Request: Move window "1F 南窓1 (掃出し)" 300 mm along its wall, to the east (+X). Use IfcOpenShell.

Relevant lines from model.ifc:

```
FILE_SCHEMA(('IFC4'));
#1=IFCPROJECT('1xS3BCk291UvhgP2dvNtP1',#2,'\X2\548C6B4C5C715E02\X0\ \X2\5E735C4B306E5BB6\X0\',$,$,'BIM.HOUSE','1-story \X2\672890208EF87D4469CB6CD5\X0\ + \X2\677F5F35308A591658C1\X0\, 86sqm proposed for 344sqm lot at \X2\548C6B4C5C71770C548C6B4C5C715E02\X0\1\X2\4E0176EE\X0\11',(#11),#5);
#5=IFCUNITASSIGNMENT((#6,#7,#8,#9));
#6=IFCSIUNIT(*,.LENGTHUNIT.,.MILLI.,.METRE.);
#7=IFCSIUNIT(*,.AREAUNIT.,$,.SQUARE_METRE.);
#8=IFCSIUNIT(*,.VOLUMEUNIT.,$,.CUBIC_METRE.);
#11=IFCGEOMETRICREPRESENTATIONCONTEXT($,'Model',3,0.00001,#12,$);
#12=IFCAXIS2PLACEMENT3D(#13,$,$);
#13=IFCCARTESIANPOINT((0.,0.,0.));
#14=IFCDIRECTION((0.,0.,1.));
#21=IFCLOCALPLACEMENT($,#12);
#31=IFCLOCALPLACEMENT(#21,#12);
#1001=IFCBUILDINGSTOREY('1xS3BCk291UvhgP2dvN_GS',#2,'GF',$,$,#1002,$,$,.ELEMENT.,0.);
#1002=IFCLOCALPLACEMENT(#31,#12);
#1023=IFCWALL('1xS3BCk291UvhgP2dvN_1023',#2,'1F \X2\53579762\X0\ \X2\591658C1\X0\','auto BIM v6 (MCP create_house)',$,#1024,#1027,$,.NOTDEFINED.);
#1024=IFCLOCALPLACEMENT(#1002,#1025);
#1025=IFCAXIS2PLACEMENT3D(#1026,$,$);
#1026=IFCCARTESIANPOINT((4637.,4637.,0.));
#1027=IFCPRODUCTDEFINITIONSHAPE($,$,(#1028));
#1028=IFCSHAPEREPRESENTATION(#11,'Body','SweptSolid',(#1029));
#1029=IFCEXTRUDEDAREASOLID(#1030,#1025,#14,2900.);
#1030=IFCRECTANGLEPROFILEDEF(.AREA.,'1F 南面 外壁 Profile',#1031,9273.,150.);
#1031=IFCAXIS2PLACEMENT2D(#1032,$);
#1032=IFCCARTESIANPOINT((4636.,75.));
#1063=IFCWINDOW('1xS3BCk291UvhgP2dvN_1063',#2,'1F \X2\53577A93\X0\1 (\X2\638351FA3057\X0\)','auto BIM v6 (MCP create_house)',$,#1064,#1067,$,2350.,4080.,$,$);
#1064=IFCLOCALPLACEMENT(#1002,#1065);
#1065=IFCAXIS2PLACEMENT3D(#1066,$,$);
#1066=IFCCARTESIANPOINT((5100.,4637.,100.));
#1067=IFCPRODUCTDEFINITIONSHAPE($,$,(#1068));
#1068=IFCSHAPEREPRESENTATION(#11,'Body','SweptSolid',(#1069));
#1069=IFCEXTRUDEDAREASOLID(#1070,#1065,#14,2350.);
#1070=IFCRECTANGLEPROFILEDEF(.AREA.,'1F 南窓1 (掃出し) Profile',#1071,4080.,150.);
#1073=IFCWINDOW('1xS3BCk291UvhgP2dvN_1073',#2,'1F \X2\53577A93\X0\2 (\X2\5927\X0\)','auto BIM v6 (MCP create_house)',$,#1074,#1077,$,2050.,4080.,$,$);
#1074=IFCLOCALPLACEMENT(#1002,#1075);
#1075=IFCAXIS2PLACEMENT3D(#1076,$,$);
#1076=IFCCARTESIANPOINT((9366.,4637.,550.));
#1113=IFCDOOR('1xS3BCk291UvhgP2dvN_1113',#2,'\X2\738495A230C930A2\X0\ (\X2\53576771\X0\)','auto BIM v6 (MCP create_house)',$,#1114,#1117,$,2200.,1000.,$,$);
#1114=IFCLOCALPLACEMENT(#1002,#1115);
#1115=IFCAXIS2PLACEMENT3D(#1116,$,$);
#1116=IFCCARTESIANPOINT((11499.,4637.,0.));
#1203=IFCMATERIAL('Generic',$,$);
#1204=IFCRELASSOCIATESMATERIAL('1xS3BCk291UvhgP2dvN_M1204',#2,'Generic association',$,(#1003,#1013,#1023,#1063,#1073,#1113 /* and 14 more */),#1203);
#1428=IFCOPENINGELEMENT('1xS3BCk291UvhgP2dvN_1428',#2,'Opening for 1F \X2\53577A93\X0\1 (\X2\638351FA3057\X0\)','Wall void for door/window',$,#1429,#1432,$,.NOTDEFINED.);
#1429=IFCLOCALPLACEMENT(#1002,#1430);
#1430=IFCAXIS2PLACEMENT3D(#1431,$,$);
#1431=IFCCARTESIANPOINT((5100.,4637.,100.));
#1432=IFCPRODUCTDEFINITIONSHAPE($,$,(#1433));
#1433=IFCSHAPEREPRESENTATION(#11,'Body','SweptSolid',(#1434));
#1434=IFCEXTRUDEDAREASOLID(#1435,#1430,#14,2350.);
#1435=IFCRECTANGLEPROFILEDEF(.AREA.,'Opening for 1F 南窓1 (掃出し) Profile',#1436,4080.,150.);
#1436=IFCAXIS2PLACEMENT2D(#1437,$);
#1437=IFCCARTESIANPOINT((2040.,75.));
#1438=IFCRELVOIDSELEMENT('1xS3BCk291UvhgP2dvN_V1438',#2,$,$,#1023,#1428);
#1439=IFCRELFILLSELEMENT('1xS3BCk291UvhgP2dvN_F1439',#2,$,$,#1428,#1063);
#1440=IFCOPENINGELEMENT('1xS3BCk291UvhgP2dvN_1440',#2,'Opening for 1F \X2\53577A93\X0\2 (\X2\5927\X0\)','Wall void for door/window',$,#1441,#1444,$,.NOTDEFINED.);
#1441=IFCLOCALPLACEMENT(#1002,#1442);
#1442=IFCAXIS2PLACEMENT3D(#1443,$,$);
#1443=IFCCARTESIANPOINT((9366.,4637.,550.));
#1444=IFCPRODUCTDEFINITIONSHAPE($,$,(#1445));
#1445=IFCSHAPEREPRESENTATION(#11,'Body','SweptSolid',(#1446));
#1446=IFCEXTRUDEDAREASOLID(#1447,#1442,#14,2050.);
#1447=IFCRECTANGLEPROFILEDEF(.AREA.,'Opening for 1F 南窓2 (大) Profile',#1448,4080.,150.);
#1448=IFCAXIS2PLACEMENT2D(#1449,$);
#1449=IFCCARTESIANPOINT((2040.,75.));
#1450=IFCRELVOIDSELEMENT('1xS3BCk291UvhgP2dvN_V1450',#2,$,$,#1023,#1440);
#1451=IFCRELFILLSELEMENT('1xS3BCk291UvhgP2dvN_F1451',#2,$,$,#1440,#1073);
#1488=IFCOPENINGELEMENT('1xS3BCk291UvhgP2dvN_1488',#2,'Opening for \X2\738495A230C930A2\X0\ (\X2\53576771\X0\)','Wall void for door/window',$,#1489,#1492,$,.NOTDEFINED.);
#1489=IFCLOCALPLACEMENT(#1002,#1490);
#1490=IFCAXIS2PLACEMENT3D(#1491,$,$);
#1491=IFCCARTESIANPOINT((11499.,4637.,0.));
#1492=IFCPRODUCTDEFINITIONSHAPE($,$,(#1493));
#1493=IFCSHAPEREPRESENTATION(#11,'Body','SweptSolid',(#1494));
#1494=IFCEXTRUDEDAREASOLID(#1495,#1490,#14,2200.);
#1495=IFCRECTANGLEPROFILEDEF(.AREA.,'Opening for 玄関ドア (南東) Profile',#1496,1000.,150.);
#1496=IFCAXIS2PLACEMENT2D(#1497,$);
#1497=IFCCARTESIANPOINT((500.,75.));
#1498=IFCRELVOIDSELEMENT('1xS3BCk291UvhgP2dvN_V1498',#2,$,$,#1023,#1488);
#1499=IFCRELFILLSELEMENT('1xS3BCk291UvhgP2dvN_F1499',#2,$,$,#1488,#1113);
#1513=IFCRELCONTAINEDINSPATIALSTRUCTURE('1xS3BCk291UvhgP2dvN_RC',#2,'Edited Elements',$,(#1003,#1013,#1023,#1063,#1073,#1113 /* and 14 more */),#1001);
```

```python
import ifcopenshell
import ifcopenshell.api.geometry
import ifcopenshell.util.placement

model = ifcopenshell.open("model.ifc")

window = model.by_guid("1xS3BCk291UvhgP2dvN_1063")
opening = window.FillsVoids[0].RelatingOpeningElement
wall = opening.VoidsElements[0].RelatingBuildingElement

wall_matrix = ifcopenshell.util.placement.get_local_placement(wall.ObjectPlacement)
shift = wall_matrix[:3, 0] * 300.0
before = ifcopenshell.util.placement.get_local_placement(window.ObjectPlacement)[:3, 3].copy()

# The window is not placed relative to its opening, so move both.
for product in (opening, window):
    matrix = ifcopenshell.util.placement.get_local_placement(product.ObjectPlacement)
    matrix[:3, 3] += shift
    ifcopenshell.api.geometry.edit_object_placement(model, product=product, matrix=matrix, is_si=False)

after = ifcopenshell.util.placement.get_local_placement(window.ObjectPlacement)[:3, 3]
print("window moved by", (after - before).round(3) + 0.0)

model.write("model_updated.ifc")
```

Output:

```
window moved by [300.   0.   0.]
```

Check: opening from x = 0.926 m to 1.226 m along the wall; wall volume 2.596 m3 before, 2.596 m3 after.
